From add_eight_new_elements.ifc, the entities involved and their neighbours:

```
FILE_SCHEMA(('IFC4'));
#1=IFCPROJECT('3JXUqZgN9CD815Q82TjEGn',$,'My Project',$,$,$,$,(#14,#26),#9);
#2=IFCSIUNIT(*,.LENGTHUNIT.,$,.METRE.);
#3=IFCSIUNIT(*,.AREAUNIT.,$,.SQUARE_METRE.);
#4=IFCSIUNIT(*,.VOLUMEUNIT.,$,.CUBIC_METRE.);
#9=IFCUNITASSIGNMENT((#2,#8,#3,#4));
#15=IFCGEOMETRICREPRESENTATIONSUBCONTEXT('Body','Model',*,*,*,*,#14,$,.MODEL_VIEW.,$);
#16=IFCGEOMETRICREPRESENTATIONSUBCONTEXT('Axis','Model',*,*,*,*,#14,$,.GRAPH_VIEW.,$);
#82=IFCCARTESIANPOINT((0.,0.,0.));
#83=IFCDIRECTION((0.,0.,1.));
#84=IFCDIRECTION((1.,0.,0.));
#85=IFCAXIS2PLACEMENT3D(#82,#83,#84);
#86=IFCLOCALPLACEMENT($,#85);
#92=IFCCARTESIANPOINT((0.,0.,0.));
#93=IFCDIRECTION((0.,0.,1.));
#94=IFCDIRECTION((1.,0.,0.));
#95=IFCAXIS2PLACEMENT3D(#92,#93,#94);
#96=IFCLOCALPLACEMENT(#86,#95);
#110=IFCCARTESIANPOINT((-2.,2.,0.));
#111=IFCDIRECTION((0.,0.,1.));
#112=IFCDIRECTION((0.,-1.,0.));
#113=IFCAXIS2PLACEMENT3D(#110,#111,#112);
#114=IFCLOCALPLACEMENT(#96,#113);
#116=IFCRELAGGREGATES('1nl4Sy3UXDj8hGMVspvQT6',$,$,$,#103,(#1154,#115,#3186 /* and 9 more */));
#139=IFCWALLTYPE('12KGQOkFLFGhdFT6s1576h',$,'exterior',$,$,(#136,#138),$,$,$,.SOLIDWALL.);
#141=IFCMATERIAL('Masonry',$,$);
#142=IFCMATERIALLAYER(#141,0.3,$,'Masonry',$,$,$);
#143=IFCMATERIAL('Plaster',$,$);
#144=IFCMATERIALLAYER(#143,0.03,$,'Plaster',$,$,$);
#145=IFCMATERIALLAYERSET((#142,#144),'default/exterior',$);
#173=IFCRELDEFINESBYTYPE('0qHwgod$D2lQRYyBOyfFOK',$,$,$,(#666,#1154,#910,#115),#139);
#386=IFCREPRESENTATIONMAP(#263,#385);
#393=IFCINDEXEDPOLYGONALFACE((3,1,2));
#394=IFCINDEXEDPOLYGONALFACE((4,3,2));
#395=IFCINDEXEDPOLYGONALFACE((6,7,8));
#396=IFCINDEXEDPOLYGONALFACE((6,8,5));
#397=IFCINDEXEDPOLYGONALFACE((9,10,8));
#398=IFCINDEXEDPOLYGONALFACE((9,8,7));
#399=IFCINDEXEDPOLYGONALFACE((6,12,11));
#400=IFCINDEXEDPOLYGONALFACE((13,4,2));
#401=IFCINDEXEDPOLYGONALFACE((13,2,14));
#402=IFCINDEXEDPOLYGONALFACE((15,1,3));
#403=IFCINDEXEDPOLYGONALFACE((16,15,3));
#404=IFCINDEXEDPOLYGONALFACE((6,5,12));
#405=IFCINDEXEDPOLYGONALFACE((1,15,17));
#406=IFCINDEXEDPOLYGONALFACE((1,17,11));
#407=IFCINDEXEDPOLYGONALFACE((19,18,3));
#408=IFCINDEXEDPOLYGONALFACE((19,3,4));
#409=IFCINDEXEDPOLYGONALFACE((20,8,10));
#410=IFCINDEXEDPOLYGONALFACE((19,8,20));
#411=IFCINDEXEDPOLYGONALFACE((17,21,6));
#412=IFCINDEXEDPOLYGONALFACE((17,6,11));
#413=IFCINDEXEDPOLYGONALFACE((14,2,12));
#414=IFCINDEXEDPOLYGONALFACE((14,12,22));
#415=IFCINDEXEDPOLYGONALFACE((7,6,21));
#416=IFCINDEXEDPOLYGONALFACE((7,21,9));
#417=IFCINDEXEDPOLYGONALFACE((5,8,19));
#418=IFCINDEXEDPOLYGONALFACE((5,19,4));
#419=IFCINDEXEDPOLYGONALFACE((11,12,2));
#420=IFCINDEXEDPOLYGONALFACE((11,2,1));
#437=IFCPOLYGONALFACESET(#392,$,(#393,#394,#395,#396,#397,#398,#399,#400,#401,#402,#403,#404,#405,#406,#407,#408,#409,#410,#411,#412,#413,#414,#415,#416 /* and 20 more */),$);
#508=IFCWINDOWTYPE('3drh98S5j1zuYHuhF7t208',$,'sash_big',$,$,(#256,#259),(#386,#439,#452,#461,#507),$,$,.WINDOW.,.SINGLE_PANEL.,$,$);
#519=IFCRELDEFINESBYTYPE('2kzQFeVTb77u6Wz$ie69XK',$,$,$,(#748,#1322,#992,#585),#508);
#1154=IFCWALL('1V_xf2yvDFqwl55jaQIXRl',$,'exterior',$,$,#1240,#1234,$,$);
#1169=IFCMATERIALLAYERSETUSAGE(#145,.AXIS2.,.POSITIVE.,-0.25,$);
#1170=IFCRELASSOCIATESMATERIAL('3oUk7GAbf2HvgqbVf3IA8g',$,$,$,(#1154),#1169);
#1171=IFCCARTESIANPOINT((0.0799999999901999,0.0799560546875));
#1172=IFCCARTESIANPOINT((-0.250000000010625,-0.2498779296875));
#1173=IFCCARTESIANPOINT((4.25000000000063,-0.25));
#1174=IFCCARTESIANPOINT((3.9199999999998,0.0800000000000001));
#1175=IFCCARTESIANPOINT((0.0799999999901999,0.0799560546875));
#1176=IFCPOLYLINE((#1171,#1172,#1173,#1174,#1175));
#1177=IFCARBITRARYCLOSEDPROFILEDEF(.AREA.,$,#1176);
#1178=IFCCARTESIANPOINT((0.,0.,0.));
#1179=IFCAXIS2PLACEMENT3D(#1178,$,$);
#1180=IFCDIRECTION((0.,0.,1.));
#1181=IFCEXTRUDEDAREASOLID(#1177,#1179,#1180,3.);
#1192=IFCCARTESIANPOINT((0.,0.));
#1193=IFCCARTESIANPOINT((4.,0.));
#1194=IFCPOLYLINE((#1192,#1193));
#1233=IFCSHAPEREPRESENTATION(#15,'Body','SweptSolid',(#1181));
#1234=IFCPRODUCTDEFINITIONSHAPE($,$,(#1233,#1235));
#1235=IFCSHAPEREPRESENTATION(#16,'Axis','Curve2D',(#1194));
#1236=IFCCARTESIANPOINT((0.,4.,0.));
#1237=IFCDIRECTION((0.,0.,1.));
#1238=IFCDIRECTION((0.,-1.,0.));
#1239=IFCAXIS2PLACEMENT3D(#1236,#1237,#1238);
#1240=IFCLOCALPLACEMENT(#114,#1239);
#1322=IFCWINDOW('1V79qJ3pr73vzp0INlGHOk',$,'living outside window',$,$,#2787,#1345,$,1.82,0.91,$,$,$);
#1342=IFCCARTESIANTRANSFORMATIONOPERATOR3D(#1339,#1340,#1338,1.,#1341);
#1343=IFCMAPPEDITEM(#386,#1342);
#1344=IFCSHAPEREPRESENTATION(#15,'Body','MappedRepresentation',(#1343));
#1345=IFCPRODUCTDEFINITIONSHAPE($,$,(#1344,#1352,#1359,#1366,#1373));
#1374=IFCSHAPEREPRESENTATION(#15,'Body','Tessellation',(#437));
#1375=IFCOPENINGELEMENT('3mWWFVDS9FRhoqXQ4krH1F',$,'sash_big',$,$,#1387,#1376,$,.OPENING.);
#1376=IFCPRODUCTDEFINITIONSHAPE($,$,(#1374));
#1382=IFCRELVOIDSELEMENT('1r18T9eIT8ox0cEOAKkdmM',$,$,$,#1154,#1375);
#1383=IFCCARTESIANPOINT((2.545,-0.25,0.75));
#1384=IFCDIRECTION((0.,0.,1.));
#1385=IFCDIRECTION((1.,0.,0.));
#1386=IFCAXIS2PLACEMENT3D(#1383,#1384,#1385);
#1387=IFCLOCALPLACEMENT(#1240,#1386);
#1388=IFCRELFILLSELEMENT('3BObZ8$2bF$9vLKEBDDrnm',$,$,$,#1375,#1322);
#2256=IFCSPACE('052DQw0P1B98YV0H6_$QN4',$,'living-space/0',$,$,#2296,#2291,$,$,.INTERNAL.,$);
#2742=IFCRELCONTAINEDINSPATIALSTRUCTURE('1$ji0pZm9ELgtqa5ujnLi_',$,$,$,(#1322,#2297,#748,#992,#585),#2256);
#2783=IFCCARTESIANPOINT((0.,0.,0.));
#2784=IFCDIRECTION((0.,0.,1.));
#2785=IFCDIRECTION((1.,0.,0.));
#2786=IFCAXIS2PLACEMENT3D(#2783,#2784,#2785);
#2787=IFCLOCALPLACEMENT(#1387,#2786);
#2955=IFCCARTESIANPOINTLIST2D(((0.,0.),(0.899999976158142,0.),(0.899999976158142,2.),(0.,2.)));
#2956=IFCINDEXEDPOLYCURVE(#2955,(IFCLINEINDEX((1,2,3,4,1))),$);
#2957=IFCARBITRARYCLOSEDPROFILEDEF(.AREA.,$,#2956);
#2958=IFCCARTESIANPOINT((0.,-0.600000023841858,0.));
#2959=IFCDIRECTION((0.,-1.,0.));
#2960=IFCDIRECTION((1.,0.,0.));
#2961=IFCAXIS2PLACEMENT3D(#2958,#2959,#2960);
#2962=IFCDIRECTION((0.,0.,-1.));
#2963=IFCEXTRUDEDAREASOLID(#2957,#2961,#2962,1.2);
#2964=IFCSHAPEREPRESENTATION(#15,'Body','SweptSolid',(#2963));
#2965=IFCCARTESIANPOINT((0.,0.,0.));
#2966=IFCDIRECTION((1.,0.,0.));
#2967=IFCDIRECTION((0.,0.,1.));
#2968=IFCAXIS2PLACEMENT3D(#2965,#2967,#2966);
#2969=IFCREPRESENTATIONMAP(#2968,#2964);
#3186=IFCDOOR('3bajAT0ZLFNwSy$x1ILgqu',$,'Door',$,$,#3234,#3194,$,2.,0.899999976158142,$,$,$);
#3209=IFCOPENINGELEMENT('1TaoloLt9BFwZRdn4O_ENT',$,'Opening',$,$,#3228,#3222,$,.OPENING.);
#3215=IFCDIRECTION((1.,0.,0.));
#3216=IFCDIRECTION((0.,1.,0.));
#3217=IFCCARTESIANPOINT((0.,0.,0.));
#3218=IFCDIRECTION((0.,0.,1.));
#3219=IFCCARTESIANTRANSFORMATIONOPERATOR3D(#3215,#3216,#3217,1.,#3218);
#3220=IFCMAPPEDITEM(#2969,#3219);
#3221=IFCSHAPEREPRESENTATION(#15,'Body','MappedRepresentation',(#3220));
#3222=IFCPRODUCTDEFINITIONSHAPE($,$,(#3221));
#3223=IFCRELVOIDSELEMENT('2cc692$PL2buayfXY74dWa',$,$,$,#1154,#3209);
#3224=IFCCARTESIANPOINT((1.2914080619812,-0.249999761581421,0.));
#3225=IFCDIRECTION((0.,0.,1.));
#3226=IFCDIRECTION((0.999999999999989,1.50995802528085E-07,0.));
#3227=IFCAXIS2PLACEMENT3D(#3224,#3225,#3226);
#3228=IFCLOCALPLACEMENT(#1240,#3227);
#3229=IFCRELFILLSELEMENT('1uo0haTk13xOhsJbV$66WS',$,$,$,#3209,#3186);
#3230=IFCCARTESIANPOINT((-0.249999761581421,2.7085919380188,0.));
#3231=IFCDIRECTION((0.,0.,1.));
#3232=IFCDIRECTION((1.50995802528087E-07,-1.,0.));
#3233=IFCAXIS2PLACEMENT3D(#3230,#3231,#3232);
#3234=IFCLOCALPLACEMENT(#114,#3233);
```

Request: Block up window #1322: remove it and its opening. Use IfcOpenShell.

```python
import ifcopenshell
import ifcopenshell.api.feature
import ifcopenshell.api.root
import ifcopenshell.geom
import ifcopenshell.util.shape

model = ifcopenshell.open("add_eight_new_elements.ifc")
settings = ifcopenshell.geom.settings()


def volume(element):
    """Net volume in cubic metres, openings subtracted."""
    shape = ifcopenshell.geom.create_shape(settings, element)
    return ifcopenshell.util.shape.get_volume(shape.geometry)


window = model.by_guid("1V79qJ3pr73vzp0INlGHOk")
opening = window.FillsVoids[0].RelatingOpeningElement
wall = opening.VoidsElements[0].RelatingBuildingElement
before = volume(wall)

ifcopenshell.api.root.remove_product(model, product=window)
ifcopenshell.api.feature.remove_feature(model, feature=opening)

after = volume(wall)

print(f"wall volume {before:.3f} -> {after:.3f} m3")

model.write("add_eight_new_elements_updated.ifc")
```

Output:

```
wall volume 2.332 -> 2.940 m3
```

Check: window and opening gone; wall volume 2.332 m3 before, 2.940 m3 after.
